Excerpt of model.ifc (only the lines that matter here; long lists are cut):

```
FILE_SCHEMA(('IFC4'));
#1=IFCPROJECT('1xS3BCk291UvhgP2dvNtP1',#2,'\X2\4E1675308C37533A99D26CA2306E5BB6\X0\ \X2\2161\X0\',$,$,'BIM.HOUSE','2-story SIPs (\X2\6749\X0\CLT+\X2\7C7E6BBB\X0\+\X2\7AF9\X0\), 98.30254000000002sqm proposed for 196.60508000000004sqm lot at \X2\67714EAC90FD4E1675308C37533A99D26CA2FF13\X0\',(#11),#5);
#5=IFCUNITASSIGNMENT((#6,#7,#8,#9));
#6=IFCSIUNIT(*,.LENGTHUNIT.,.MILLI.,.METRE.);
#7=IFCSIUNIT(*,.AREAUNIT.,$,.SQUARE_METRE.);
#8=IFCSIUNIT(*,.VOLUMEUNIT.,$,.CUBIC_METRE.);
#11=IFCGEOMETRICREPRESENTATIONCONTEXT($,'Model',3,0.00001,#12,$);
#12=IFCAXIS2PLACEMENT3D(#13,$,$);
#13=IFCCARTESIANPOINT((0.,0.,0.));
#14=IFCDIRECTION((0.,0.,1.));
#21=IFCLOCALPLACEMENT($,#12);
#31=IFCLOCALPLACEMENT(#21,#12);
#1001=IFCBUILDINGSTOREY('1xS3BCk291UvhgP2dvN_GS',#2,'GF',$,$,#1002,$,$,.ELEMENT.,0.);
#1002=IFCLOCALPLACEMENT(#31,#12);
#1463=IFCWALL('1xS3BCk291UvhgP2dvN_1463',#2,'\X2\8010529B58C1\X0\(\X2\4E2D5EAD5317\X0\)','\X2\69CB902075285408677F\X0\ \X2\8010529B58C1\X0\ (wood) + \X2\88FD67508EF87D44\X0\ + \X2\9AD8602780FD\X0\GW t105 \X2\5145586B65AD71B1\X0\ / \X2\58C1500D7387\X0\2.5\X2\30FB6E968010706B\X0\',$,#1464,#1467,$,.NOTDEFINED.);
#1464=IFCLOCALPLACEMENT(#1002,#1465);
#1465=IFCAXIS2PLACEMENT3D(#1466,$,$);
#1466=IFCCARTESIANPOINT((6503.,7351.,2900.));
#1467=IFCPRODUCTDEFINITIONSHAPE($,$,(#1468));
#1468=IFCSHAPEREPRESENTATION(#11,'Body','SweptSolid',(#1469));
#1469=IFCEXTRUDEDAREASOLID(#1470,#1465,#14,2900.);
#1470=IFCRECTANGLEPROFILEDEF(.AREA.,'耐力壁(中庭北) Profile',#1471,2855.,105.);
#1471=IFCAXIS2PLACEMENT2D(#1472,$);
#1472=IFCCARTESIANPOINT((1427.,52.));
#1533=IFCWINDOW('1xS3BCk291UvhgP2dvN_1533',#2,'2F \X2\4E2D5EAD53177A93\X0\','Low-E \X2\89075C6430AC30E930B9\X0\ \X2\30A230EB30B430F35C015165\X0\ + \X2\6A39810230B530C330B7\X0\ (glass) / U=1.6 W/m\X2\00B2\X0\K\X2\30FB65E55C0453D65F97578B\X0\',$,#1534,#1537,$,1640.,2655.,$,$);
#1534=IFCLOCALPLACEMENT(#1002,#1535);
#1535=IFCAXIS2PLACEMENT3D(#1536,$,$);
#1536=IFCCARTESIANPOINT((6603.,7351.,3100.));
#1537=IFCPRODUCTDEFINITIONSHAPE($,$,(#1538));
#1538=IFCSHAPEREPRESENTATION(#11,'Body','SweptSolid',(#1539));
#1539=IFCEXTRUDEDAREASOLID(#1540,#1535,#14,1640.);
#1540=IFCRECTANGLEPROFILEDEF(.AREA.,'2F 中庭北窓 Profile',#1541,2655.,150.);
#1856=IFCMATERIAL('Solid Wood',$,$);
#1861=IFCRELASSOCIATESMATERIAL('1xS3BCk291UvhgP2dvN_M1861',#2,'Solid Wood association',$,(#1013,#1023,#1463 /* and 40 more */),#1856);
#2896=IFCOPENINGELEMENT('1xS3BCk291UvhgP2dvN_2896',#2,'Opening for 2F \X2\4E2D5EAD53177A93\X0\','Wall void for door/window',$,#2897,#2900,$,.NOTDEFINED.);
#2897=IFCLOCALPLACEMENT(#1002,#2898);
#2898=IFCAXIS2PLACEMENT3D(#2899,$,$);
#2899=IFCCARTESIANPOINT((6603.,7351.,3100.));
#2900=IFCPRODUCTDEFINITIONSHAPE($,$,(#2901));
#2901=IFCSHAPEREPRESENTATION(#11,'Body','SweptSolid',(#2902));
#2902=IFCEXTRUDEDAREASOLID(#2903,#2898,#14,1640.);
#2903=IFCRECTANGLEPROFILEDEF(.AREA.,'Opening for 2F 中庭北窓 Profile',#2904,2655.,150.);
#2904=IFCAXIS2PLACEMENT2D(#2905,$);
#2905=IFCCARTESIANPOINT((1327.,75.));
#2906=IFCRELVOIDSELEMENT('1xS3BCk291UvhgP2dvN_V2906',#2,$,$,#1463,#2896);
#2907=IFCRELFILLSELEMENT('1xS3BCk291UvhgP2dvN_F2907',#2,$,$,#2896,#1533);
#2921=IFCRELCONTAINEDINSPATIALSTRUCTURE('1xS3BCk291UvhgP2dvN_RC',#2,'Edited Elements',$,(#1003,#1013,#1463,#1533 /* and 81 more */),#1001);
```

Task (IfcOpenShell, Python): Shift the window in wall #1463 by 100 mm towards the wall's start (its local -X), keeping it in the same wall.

```python
import ifcopenshell
import ifcopenshell.api.geometry
import ifcopenshell.util.placement

model = ifcopenshell.open("model.ifc")

window = model.by_guid("1xS3BCk291UvhgP2dvN_1533")
opening = window.FillsVoids[0].RelatingOpeningElement
wall = opening.VoidsElements[0].RelatingBuildingElement

wall_matrix = ifcopenshell.util.placement.get_local_placement(wall.ObjectPlacement)
shift = wall_matrix[:3, 0] * -100.0
before = ifcopenshell.util.placement.get_local_placement(window.ObjectPlacement)[:3, 3].copy()

# The window is not placed relative to its opening, so move both.
for product in (opening, window):
    matrix = ifcopenshell.util.placement.get_local_placement(product.ObjectPlacement)
    matrix[:3, 3] += shift
    ifcopenshell.api.geometry.edit_object_placement(model, product=product, matrix=matrix, is_si=False)

after = ifcopenshell.util.placement.get_local_placement(window.ObjectPlacement)[:3, 3]
print("window moved by", (after - before).round(3) + 0.0)

model.write("model_v2.ifc")
```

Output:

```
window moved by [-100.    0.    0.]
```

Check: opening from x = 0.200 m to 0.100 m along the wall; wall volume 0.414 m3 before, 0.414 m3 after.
